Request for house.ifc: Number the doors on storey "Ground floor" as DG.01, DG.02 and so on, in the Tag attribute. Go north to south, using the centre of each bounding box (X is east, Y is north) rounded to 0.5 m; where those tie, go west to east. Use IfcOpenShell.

First a look at what the model holds.

```python
import ifcopenshell
import ifcopenshell.util.element
import ifcopenshell.util.placement

model = ifcopenshell.open("house.ifc")
print(model.schema)
storey = next(s for s in model.by_type("IfcBuildingStorey") if s.Name == "Ground floor")
doors = [e for e in ifcopenshell.util.element.get_decomposition(storey) if e.is_a("IfcDoor")]
for e in sorted(doors, key=lambda e: e.id()):
    origin = ifcopenshell.util.placement.get_local_placement(e.ObjectPlacement)[:3, 3]
    print(e.id(), e.Tag, e.Name, origin.round(2) + 0.0, sep=" | ")
```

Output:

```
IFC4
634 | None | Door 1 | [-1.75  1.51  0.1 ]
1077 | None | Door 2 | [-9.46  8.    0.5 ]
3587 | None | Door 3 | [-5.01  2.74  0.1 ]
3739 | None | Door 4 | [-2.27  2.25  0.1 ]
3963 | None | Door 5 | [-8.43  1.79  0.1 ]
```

```python
import ifcopenshell
import ifcopenshell.geom
import ifcopenshell.util.element
import ifcopenshell.util.shape

model = ifcopenshell.open("house.ifc")
settings = ifcopenshell.geom.settings()
settings.set("use-world-coords", True)


def centre(element):
    shape = ifcopenshell.geom.create_shape(settings, element)
    return ifcopenshell.util.shape.get_bbox_centroid(shape.geometry)


storey = next(s for s in model.by_type("IfcBuildingStorey") if s.Name == "Ground floor")
doors = [e for e in ifcopenshell.util.element.get_decomposition(storey) if e.is_a("IfcDoor")]

# Insertion points can sit at a corner or the storey origin, so sort by the geometry (in metres).
centres = {e: centre(e) for e in doors}
doors.sort(key=lambda e: (-round(centres[e][1] / 0.5), centres[e][0]))

for i, e in enumerate(doors, start=1):
    number = f"DG.{i:02d}"
    e.Tag = number
    print(e.id(), number)

model.write("house_edited.ifc")
```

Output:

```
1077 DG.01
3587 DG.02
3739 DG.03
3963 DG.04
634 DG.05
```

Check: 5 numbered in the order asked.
